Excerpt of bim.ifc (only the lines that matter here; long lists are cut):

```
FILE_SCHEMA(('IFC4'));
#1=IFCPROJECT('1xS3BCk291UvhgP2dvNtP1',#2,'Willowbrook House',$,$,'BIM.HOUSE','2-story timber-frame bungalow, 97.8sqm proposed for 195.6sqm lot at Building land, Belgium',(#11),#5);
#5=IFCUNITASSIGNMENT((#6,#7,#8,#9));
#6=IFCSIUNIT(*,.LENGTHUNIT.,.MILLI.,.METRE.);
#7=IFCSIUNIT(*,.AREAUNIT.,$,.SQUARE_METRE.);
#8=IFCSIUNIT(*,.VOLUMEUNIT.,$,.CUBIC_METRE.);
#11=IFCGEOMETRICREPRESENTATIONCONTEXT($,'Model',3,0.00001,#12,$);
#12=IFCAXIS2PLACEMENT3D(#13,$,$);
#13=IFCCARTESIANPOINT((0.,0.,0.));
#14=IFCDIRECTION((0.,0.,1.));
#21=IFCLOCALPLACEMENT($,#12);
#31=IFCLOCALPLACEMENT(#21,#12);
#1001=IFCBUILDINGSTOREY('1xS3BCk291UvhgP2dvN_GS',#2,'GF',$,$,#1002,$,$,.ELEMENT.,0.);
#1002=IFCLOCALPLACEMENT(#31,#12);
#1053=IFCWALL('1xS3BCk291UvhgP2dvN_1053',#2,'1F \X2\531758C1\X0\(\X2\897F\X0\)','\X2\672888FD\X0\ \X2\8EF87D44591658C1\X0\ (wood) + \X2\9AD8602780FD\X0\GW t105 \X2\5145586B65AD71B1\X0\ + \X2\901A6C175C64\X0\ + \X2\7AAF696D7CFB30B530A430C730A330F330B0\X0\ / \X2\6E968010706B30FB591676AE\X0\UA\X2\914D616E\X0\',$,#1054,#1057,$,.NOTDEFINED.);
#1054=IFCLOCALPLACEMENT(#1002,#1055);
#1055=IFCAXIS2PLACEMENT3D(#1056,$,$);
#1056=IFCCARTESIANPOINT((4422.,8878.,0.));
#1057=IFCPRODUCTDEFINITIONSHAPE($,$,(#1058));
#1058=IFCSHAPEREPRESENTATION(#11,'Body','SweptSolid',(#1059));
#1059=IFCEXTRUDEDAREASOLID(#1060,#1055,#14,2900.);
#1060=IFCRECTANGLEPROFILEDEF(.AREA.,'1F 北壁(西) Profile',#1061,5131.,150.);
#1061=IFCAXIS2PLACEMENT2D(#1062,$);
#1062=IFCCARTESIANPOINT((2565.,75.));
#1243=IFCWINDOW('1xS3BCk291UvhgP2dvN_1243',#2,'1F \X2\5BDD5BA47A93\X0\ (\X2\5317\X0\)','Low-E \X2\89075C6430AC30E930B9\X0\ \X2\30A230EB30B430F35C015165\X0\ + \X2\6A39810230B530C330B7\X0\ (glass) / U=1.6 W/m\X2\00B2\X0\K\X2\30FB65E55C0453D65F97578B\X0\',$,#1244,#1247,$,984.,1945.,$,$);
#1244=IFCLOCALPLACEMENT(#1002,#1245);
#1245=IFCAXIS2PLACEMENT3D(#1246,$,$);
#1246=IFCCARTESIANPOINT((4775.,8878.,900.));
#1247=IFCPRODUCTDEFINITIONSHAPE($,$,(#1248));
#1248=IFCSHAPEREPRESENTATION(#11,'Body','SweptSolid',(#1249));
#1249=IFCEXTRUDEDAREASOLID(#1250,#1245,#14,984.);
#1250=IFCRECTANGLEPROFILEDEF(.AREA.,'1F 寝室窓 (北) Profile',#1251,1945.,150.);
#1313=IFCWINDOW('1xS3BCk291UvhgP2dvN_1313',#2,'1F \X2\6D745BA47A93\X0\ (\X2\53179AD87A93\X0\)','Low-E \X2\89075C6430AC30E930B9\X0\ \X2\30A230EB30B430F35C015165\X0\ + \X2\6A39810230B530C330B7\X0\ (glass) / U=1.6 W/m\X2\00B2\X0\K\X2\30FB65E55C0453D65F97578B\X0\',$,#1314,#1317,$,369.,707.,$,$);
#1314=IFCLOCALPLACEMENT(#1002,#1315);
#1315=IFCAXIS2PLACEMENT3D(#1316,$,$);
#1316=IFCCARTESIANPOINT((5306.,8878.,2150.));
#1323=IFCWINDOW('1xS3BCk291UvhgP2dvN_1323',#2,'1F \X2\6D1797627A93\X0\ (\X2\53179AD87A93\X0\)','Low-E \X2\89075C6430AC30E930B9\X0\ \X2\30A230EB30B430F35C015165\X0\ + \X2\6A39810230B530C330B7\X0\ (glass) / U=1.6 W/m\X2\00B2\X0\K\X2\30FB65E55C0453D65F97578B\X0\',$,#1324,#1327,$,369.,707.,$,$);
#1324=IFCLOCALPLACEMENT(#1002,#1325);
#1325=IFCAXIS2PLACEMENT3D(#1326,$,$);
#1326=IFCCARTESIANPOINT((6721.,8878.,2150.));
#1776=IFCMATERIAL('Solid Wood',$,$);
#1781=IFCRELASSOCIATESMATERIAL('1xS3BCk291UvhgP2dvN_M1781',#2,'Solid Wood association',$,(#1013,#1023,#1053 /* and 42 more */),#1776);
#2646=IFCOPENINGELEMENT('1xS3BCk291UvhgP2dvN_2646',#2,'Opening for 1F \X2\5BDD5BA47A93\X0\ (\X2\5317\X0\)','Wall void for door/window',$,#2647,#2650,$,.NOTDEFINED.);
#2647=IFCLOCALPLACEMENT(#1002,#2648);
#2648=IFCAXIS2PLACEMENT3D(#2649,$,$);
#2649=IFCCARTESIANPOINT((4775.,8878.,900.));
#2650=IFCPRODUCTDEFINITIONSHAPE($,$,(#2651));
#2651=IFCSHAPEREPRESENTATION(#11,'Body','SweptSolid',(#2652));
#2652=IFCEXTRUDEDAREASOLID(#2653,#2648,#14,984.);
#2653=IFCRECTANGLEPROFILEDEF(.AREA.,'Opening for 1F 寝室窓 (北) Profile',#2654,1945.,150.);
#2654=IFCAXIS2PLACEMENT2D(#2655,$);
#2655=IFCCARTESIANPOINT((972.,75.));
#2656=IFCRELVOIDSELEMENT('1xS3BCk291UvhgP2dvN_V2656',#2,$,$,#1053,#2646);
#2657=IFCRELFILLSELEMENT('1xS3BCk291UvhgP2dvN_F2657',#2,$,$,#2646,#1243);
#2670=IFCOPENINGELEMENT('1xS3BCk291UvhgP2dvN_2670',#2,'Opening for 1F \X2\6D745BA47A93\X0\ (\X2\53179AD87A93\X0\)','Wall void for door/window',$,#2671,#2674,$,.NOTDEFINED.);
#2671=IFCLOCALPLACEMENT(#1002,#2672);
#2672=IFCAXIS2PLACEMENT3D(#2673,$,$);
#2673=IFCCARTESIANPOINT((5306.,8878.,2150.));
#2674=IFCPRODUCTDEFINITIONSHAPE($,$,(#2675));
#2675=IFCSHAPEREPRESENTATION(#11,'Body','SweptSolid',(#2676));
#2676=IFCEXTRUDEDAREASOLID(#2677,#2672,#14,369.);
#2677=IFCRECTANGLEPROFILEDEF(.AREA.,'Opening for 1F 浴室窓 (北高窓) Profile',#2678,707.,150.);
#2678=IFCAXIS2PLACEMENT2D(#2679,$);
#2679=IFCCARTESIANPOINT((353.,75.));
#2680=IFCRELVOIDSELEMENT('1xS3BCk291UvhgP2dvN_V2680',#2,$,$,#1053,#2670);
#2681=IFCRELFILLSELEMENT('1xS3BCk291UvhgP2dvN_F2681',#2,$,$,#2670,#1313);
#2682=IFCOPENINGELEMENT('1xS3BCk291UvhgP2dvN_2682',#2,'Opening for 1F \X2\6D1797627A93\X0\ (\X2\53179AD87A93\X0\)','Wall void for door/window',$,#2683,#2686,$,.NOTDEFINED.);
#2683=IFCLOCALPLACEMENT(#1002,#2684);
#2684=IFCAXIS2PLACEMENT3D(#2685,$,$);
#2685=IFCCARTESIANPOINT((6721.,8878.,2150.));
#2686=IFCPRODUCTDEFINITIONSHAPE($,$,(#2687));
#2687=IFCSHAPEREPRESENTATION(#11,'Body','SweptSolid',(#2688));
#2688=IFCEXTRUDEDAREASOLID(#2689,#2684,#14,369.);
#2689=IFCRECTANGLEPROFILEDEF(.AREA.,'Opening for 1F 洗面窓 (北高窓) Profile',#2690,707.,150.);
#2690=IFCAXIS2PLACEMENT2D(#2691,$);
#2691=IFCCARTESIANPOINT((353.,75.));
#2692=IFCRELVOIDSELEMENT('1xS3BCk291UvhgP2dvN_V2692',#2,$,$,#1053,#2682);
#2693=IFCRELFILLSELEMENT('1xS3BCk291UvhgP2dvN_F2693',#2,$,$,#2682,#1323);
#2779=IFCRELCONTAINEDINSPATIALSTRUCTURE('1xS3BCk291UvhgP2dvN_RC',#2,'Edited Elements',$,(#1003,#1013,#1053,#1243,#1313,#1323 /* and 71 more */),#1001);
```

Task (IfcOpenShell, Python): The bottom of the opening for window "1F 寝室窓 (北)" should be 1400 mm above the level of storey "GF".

```python
import numpy as np
import ifcopenshell
import ifcopenshell.api.geometry
import ifcopenshell.geom
import ifcopenshell.util.element
import ifcopenshell.util.placement
import ifcopenshell.util.shape
import ifcopenshell.util.unit

model = ifcopenshell.open("bim.ifc")
unit_scale = ifcopenshell.util.unit.calculate_unit_scale(model)

window = model.by_guid("1xS3BCk291UvhgP2dvN_1243")
opening = window.FillsVoids[0].RelatingOpeningElement
storey = ifcopenshell.util.element.get_container(window, ifc_class="IfcBuildingStorey")
level = ifcopenshell.util.placement.get_local_placement(storey.ObjectPlacement)[2, 3]

# The opening's origin need not be at the sill, so measure its lowest point.
shape = ifcopenshell.geom.create_shape(ifcopenshell.geom.settings(), opening)
bottom = ifcopenshell.util.shape.get_shape_bottom_elevation(shape, shape.geometry) / unit_scale
dz = level + 1.4 / unit_scale - bottom

shift = np.array([0.0, 0.0, dz])
# The window is not placed relative to its opening, so move both.
for product in (opening, window):
    matrix = ifcopenshell.util.placement.get_local_placement(product.ObjectPlacement)
    matrix[:3, 3] += shift
    ifcopenshell.api.geometry.edit_object_placement(model, product=product, matrix=matrix, is_si=False)

print(f"moved by {dz * unit_scale:+.3f} m")

model.write("bim_rev.ifc")
```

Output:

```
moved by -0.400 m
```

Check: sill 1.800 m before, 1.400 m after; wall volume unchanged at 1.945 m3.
